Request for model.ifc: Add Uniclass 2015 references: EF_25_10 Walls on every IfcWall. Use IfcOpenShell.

First a look at what the model holds.

```python
import ifcopenshell

model = ifcopenshell.open("model.ifc")
print(model.schema)
print("classifications:", [c.Name for c in model.by_type("IfcClassification")])
for ifc_class in ("IfcDoor", "IfcRoof", "IfcStair", "IfcWall", "IfcWindow"):
    print(ifc_class, len(model.by_type(ifc_class)))
```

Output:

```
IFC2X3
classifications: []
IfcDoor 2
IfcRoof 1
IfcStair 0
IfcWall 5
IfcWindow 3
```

```python
import ifcopenshell
import ifcopenshell.api.classification

model = ifcopenshell.open("model.ifc")

# IFC2X3 requires Source and Edition and has no link from the project to the system.
system = model.create_entity("IfcClassification", Source="NBS", Edition="2015", Name="Uniclass 2015")

codes = {
    "IfcWall": ("EF_25_10", "Walls"),
}
for ifc_class, (code, name) in codes.items():
    products = model.by_type(ifc_class)
    ifcopenshell.api.classification.add_reference(
        model, products=products, classification=system, identification=code, name=name
    )
    print(code, len(products))

model.write("model-out.ifc")
```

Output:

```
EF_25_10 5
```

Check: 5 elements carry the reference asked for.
